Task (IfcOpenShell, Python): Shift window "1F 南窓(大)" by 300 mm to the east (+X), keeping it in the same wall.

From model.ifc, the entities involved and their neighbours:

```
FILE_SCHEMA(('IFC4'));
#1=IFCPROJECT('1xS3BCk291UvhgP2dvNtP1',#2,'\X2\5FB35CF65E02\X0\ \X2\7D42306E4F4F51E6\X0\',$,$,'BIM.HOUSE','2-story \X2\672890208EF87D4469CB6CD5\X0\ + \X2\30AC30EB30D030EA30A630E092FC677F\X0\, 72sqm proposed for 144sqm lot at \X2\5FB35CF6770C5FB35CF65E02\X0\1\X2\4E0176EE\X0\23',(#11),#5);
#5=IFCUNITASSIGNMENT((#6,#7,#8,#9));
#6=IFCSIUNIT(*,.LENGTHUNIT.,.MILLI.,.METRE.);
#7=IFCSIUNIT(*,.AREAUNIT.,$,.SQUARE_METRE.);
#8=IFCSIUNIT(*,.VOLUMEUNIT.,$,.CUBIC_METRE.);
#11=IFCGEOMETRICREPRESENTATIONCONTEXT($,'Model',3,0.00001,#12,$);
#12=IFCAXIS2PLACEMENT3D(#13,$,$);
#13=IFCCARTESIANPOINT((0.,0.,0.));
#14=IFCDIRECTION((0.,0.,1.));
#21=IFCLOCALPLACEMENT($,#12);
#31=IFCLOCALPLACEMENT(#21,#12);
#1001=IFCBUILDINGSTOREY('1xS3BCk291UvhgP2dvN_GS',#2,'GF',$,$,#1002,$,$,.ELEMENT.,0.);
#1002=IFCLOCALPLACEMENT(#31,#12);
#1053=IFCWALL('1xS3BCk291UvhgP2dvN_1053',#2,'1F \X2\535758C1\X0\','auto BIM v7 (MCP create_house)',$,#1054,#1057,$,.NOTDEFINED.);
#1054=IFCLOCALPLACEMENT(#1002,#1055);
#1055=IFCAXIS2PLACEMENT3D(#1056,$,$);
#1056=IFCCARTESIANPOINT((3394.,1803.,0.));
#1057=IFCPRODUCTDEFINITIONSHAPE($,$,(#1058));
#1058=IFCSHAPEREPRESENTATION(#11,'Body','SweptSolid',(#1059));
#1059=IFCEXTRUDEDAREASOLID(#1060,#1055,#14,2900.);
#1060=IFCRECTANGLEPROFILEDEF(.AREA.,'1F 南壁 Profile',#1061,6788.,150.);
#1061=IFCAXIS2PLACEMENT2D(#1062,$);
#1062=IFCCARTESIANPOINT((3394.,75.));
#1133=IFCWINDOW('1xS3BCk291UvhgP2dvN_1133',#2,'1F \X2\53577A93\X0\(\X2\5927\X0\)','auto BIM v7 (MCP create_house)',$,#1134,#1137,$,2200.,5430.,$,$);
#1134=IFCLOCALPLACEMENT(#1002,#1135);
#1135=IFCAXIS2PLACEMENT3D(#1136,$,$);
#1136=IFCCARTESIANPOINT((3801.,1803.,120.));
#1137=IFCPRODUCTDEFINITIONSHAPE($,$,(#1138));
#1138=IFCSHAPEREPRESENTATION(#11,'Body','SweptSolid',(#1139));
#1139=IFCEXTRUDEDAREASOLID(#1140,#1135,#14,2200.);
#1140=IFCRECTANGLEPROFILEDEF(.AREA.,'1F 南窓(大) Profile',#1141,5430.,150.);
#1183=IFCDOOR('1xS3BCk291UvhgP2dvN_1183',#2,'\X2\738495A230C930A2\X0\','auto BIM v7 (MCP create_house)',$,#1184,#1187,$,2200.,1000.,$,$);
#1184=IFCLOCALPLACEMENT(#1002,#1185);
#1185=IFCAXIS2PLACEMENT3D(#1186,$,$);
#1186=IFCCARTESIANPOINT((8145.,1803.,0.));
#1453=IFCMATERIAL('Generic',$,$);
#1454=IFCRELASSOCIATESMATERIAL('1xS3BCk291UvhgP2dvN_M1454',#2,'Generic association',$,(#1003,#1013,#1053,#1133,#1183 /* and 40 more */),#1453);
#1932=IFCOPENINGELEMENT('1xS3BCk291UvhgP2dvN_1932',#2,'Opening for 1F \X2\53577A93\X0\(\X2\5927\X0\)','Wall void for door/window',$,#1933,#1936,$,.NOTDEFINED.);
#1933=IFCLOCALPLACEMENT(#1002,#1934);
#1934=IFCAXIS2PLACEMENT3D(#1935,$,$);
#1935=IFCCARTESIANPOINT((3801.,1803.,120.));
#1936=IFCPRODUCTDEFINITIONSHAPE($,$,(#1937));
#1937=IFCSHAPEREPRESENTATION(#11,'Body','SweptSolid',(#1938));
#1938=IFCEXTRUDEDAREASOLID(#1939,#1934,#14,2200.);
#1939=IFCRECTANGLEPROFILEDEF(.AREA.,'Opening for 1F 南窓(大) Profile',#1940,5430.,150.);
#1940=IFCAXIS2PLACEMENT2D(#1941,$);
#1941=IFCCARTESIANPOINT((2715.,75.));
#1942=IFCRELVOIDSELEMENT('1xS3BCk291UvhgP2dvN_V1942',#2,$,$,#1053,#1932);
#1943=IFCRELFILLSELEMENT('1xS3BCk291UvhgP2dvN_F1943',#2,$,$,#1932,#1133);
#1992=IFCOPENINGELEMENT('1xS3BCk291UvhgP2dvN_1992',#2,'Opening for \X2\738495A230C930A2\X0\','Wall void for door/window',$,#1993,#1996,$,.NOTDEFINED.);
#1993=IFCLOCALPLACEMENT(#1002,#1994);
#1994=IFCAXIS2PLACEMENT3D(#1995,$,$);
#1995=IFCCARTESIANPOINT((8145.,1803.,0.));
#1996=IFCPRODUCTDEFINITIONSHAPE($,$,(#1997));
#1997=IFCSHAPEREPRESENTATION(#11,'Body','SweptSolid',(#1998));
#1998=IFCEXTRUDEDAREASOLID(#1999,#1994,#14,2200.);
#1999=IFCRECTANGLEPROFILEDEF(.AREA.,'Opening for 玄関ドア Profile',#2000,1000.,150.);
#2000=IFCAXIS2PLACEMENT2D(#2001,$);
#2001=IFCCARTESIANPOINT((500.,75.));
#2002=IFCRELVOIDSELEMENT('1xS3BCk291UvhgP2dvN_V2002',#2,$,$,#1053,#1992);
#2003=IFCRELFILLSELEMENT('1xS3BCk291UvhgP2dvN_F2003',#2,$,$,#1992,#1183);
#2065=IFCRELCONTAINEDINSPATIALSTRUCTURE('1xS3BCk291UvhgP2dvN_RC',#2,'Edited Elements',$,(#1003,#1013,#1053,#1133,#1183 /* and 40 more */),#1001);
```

```python
import ifcopenshell
import ifcopenshell.api.geometry
import ifcopenshell.util.placement
import ifcopenshell.util.unit

model = ifcopenshell.open("model.ifc")
unit_scale = ifcopenshell.util.unit.calculate_unit_scale(model)

window = model.by_guid("1xS3BCk291UvhgP2dvN_1133")
opening = window.FillsVoids[0].RelatingOpeningElement
wall = opening.VoidsElements[0].RelatingBuildingElement

wall_matrix = ifcopenshell.util.placement.get_local_placement(wall.ObjectPlacement)
shift = wall_matrix[:3, 0] * 0.3 / unit_scale
before = ifcopenshell.util.placement.get_local_placement(window.ObjectPlacement)[:3, 3].copy()

# The window is not placed relative to its opening, so move both.
for product in (opening, window):
    matrix = ifcopenshell.util.placement.get_local_placement(product.ObjectPlacement)
    matrix[:3, 3] += shift
    ifcopenshell.api.geometry.edit_object_placement(model, product=product, matrix=matrix, is_si=False)

after = ifcopenshell.util.placement.get_local_placement(window.ObjectPlacement)[:3, 3]
print("window moved by", (after - before).round(3) + 0.0)

model.write("model_edited.ifc")
```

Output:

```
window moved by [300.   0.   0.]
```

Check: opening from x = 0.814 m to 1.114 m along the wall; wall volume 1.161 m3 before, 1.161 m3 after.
